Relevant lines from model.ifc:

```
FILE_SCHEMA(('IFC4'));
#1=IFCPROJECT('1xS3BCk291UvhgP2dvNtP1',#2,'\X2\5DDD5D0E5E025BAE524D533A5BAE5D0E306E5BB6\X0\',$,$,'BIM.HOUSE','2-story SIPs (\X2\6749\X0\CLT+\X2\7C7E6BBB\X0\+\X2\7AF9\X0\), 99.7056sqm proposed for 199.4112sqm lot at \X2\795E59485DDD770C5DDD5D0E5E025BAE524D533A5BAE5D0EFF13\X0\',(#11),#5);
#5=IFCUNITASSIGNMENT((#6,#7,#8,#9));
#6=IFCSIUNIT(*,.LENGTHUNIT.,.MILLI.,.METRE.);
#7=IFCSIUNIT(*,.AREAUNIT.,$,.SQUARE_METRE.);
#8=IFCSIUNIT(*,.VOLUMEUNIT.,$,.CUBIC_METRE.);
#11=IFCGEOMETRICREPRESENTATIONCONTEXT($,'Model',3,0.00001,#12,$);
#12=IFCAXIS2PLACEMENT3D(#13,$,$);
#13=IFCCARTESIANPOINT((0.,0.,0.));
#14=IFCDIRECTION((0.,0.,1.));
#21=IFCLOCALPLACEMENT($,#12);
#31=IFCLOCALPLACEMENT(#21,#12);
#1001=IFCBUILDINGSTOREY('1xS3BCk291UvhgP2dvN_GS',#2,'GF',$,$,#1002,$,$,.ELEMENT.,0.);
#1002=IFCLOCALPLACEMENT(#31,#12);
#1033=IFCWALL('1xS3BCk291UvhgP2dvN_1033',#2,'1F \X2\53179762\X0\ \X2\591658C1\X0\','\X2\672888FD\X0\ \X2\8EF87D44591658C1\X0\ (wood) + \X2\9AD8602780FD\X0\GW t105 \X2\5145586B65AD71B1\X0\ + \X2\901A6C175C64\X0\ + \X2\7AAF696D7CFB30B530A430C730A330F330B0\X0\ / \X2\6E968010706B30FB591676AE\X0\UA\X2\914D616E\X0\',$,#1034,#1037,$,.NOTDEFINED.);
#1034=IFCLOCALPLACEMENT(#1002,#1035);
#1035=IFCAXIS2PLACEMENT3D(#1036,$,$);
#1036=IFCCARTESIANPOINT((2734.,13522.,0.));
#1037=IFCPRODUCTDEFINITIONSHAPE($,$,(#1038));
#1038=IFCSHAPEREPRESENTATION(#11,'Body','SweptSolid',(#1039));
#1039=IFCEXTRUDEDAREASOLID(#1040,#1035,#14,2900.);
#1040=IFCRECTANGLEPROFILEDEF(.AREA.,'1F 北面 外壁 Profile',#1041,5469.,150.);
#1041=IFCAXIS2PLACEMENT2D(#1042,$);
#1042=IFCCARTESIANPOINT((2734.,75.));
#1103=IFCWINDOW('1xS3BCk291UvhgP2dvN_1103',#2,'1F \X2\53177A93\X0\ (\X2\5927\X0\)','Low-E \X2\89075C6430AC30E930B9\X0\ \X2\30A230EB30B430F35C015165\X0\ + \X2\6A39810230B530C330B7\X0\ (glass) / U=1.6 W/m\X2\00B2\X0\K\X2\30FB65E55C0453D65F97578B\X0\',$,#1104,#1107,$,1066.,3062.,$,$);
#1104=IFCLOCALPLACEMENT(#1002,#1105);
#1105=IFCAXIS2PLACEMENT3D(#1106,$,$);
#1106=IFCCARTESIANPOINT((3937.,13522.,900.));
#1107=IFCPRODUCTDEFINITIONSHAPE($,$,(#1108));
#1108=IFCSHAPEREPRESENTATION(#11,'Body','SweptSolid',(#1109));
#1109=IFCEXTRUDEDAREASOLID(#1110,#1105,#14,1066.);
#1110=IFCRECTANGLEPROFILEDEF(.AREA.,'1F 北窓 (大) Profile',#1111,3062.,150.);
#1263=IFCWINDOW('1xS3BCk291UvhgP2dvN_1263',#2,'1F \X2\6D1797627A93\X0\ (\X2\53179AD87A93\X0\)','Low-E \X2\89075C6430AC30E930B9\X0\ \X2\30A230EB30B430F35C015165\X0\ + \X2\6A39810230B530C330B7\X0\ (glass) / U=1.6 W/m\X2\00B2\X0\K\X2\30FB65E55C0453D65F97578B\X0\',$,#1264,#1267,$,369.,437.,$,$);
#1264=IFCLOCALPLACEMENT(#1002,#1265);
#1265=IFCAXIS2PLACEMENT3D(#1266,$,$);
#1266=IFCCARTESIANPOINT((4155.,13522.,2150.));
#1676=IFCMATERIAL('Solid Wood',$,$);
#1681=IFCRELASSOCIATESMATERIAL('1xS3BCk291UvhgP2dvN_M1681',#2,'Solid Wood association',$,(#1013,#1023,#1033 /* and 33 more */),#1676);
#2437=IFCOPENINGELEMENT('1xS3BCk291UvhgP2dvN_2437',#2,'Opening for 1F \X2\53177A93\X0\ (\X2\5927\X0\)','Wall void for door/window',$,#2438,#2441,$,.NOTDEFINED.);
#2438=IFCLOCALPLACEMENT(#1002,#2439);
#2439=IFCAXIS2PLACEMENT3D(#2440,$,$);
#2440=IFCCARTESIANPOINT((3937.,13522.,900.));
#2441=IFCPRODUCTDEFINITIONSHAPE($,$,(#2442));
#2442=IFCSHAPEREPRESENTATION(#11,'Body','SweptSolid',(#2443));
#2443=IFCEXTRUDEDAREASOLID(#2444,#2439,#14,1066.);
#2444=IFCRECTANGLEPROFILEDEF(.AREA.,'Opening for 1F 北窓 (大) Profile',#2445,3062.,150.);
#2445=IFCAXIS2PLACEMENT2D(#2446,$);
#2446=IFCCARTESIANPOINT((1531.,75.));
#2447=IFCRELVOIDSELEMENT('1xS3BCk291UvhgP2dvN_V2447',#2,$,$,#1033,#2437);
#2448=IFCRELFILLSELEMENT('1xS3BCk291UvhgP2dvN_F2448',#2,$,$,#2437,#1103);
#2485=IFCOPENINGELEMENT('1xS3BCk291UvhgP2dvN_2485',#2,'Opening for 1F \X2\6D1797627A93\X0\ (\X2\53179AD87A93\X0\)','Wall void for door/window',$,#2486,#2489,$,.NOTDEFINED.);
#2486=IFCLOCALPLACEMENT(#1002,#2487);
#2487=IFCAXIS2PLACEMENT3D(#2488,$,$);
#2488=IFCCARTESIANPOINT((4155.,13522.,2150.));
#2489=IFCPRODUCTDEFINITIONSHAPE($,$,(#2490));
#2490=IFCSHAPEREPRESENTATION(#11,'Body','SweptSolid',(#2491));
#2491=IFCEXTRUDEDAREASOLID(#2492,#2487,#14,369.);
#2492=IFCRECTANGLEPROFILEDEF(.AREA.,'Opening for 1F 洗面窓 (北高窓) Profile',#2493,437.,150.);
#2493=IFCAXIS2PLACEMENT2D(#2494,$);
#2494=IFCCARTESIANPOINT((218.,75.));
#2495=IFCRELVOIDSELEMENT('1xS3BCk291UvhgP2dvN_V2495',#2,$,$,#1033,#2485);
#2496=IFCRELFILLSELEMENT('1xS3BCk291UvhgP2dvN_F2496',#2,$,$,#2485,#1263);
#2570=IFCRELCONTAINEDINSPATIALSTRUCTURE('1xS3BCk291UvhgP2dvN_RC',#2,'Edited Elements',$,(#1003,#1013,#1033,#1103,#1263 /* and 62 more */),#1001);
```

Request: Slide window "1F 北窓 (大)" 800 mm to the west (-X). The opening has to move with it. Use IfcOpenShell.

```python
import ifcopenshell
import ifcopenshell.api.geometry
import ifcopenshell.util.placement
import ifcopenshell.util.unit

model = ifcopenshell.open("model.ifc")
unit_scale = ifcopenshell.util.unit.calculate_unit_scale(model)

window = model.by_guid("1xS3BCk291UvhgP2dvN_1103")
opening = window.FillsVoids[0].RelatingOpeningElement
wall = opening.VoidsElements[0].RelatingBuildingElement

wall_matrix = ifcopenshell.util.placement.get_local_placement(wall.ObjectPlacement)
shift = wall_matrix[:3, 0] * -0.8 / unit_scale
before = ifcopenshell.util.placement.get_local_placement(window.ObjectPlacement)[:3, 3].copy()

# The window is not placed relative to its opening, so move both.
for product in (opening, window):
    matrix = ifcopenshell.util.placement.get_local_placement(product.ObjectPlacement)
    matrix[:3, 3] += shift
    ifcopenshell.api.geometry.edit_object_placement(model, product=product, matrix=matrix, is_si=False)

after = ifcopenshell.util.placement.get_local_placement(window.ObjectPlacement)[:3, 3]
print("window moved by", (after - before).round(3) + 0.0)

model.write("model-out.ifc")
```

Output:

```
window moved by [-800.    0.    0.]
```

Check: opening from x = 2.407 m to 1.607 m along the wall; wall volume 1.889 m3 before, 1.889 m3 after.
